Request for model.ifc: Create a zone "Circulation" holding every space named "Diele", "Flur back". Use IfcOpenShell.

First a look at what the model holds.

```python
import ifcopenshell

model = ifcopenshell.open("model.ifc")
print(model.schema)
seen = {}
for space in model.by_type("IfcSpace"):
    seen[space.LongName] = seen.get(space.LongName, 0) + 1
for name, count in sorted(seen.items(), key=str):
    print(count, "x", name)
print("zones:", [z.Name for z in model.by_type("IfcZone")][:20])
```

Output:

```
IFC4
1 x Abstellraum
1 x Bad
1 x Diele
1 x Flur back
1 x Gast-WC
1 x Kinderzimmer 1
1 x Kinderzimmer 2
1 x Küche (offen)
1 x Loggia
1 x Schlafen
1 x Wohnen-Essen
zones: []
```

```python
import ifcopenshell
import ifcopenshell.api.group
import ifcopenshell.api.root

model = ifcopenshell.open("model.ifc")

names = {"Diele", "Flur back"}
spaces = [s for s in model.by_type("IfcSpace") if s.LongName in names]

zone = ifcopenshell.api.root.create_entity(model, ifc_class="IfcZone", name="Circulation")
ifcopenshell.api.group.assign_group(model, products=spaces, group=zone)
print(len(spaces), "spaces in", zone.Name)

model.write("model_edited.ifc")
```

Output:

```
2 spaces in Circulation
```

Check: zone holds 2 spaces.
